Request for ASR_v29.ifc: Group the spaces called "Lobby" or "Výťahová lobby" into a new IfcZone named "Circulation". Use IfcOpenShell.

First a look at what the model holds.

```python
import ifcopenshell

model = ifcopenshell.open("ASR_v29.ifc")
print(model.schema)
seen = {}
for space in model.by_type("IfcSpace"):
    seen[space.LongName] = seen.get(space.LongName, 0) + 1
for name, count in sorted(seen.items(), key=str):
    print(count, "x", name)
print("zones:", [z.Name for z in model.by_type("IfcZone")][:20])
```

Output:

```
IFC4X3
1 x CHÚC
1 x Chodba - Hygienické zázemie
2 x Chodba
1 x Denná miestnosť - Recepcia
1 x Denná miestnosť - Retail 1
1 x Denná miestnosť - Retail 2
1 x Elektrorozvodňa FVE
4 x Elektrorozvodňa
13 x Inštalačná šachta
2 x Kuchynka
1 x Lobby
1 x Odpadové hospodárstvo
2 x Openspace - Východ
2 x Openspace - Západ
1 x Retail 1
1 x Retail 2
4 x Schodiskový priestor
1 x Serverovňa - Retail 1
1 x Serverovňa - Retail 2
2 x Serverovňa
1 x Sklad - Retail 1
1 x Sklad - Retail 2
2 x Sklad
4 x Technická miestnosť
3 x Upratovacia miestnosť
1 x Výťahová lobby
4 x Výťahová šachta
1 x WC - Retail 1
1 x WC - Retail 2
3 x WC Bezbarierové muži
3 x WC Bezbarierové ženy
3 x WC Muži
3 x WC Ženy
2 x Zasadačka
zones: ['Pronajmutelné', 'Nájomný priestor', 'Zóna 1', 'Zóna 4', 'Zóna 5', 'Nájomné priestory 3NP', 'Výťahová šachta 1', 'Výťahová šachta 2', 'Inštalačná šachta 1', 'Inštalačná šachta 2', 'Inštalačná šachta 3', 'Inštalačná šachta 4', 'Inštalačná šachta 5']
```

```python
import ifcopenshell
import ifcopenshell.api.group
import ifcopenshell.api.root

model = ifcopenshell.open("ASR_v29.ifc")

names = {"Lobby", "Výťahová lobby"}
spaces = [s for s in model.by_type("IfcSpace") if s.LongName in names]

zone = ifcopenshell.api.root.create_entity(model, ifc_class="IfcZone", name="Circulation")
ifcopenshell.api.group.assign_group(model, products=spaces, group=zone)
print(len(spaces), "spaces in", zone.Name)

model.write("ASR_v29_v2.ifc")
```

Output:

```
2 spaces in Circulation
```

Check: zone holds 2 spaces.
